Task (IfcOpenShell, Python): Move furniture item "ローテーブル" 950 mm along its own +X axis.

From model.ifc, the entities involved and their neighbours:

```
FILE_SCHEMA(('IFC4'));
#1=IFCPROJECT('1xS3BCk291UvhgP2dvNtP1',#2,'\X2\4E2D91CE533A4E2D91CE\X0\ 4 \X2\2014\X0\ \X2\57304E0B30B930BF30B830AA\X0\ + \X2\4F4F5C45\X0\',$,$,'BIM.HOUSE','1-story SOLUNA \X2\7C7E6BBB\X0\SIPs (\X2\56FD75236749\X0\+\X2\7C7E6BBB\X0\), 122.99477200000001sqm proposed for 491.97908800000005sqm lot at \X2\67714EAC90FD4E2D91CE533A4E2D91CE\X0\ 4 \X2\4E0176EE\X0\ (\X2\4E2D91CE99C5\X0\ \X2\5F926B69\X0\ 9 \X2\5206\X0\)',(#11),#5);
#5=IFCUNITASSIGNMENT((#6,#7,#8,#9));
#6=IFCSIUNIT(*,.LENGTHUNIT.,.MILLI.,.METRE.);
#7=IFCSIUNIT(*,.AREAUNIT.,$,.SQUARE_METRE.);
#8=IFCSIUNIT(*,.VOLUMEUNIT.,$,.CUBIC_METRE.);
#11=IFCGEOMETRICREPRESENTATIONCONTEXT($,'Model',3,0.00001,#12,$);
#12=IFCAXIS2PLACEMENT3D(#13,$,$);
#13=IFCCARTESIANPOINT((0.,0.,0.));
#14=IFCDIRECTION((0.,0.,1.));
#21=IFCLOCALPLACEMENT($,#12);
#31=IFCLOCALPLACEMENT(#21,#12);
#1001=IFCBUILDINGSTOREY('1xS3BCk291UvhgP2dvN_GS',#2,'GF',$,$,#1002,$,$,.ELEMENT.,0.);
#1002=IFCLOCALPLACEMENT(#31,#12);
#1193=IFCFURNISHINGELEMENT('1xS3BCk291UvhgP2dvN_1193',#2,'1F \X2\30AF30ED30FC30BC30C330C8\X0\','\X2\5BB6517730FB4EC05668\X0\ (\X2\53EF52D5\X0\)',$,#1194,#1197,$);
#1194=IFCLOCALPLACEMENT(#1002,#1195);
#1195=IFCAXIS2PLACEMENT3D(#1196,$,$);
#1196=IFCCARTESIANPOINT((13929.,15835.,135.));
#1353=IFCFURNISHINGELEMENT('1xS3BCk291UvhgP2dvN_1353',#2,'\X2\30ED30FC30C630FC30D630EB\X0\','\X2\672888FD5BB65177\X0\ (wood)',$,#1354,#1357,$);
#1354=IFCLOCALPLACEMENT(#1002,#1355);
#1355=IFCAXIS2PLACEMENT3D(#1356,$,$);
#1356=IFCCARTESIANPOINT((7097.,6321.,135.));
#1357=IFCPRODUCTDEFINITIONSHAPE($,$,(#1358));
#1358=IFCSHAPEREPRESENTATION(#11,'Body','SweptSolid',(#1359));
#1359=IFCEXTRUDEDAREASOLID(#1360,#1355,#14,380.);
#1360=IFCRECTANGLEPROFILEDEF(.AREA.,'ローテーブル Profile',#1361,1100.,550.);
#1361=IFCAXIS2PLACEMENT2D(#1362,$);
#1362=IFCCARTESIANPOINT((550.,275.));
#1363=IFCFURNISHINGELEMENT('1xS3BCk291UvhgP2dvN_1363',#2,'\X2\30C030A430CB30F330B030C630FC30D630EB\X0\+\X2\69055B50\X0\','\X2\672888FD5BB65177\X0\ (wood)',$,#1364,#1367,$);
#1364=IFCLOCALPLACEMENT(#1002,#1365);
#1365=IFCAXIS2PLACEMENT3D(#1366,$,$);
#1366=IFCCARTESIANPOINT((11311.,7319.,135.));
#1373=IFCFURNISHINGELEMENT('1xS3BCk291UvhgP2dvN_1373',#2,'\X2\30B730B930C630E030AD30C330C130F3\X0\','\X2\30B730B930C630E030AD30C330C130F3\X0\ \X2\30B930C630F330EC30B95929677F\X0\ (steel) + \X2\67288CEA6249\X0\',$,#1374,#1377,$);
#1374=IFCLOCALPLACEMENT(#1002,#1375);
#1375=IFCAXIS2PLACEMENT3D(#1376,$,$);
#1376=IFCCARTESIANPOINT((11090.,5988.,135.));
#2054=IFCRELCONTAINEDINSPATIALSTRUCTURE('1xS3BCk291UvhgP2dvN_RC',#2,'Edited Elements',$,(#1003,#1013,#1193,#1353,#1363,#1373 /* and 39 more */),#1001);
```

```python
import ifcopenshell
import ifcopenshell.api.geometry
import ifcopenshell.util.placement
import ifcopenshell.util.unit

model = ifcopenshell.open("model.ifc")
unit_scale = ifcopenshell.util.unit.calculate_unit_scale(model)

item = model.by_guid("1xS3BCk291UvhgP2dvN_1353")
matrix = ifcopenshell.util.placement.get_local_placement(item.ObjectPlacement)
matrix[:3, 3] += matrix[:3, 0] * 0.95 / unit_scale
ifcopenshell.api.geometry.edit_object_placement(model, product=item, matrix=matrix, is_si=False)

print(ifcopenshell.util.placement.get_local_placement(item.ObjectPlacement).round(3) + 0.0)

model.write("model-out.ifc")
```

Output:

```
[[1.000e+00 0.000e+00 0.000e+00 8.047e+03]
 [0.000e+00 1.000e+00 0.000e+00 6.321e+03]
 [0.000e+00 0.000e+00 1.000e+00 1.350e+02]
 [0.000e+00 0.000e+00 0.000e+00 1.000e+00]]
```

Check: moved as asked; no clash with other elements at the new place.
